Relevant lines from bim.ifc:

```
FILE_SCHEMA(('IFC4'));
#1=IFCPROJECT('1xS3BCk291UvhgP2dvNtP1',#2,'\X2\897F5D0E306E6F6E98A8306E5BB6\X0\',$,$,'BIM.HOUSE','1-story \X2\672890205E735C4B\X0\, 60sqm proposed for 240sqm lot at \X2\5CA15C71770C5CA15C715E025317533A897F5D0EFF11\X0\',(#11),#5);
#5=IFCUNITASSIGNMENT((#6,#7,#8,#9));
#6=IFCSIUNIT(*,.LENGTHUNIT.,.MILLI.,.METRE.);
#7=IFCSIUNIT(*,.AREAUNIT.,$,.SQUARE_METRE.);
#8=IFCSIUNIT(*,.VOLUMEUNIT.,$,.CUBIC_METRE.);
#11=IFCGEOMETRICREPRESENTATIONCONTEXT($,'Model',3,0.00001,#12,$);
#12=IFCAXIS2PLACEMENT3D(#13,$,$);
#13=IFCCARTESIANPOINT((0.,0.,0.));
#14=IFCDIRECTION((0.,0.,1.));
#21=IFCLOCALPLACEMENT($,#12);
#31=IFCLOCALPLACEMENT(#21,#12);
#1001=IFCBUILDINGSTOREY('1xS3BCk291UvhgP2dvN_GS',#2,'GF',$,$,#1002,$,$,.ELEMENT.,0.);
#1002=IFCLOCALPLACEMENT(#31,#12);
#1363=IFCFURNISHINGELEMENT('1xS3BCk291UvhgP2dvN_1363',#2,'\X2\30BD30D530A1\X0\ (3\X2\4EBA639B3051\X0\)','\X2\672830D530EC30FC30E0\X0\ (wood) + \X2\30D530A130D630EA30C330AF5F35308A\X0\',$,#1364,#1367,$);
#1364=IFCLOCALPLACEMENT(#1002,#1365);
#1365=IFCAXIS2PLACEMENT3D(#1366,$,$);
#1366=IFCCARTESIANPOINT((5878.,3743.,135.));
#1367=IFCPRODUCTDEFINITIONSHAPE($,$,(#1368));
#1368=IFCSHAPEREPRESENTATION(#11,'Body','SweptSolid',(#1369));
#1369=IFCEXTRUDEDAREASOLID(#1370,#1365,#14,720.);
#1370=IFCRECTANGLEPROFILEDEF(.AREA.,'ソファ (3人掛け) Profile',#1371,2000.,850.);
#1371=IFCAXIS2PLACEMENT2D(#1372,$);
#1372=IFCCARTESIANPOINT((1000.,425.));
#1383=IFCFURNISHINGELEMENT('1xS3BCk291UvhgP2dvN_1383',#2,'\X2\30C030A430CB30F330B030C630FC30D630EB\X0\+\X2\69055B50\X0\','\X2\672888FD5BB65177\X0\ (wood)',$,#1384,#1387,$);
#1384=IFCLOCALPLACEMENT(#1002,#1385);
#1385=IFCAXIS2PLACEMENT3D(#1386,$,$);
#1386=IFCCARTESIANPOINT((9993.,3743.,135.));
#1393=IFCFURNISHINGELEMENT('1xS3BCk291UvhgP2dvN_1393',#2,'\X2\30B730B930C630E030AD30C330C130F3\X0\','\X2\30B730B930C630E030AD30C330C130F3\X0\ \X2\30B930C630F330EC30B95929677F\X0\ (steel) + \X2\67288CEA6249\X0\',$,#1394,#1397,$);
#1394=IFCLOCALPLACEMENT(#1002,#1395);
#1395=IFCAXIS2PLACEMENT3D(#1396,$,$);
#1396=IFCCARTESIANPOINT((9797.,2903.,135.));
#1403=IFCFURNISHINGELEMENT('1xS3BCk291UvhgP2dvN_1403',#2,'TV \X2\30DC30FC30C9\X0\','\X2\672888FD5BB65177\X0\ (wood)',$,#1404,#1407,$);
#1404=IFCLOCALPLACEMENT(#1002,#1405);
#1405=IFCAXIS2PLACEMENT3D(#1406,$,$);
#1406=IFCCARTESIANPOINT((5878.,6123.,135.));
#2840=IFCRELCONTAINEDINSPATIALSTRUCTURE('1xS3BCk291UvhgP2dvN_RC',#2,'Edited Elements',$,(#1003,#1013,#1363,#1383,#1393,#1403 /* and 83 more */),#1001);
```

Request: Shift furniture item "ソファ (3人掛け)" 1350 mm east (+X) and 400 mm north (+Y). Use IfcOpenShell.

```python
import ifcopenshell
import ifcopenshell.api.geometry
import ifcopenshell.util.placement
import ifcopenshell.util.unit

model = ifcopenshell.open("bim.ifc")
unit_scale = ifcopenshell.util.unit.calculate_unit_scale(model)

item = model.by_guid("1xS3BCk291UvhgP2dvN_1363")
matrix = ifcopenshell.util.placement.get_local_placement(item.ObjectPlacement)
matrix[0, 3] += 1.35 / unit_scale
matrix[1, 3] += 0.4 / unit_scale
ifcopenshell.api.geometry.edit_object_placement(model, product=item, matrix=matrix, is_si=False)

print(ifcopenshell.util.placement.get_local_placement(item.ObjectPlacement).round(3) + 0.0)

model.write("bim_rev.ifc")
```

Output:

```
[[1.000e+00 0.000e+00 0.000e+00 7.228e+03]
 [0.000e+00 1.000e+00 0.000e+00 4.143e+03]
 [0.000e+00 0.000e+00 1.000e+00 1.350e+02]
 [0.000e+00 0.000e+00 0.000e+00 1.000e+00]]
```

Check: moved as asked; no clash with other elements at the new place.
